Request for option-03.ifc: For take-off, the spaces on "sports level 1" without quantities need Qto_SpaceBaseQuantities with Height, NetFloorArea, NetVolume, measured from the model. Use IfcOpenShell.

First a look at what the model holds.

```python
import ifcopenshell
import ifcopenshell.util.element
import ifcopenshell.util.unit

model = ifcopenshell.open("option-03.ifc")
print(model.schema)
for unit_type in ("LENGTHUNIT", "AREAUNIT", "VOLUMEUNIT"):
    print(unit_type, ifcopenshell.util.unit.calculate_unit_scale(model, unit_type))
storey = next(s for s in model.by_type("IfcBuildingStorey") if s.Name == "sports level 1")
spaces = [e for e in ifcopenshell.util.element.get_decomposition(storey) if e.is_a("IfcSpace")]
for e in sorted(spaces, key=lambda e: e.id()):
    print(e.id(), e.is_a(), e.Name, list(ifcopenshell.util.element.get_psets(e, qtos_only=True)), sep=" | ")
```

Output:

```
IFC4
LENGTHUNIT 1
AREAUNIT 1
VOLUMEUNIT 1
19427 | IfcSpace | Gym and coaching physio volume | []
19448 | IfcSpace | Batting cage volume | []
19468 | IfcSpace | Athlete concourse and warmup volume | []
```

```python
import ifcopenshell
import ifcopenshell.api.pset
import ifcopenshell.geom
import ifcopenshell.util.element
import ifcopenshell.util.shape
import ifcopenshell.util.unit

model = ifcopenshell.open("option-03.ifc")
unit_scale = ifcopenshell.util.unit.calculate_unit_scale(model)
area_scale = ifcopenshell.util.unit.calculate_unit_scale(model, "AREAUNIT")
volume_scale = ifcopenshell.util.unit.calculate_unit_scale(model, "VOLUMEUNIT")
settings = ifcopenshell.geom.settings()

storey = next(s for s in model.by_type("IfcBuildingStorey") if s.Name == "sports level 1")
spaces = [e for e in ifcopenshell.util.element.get_decomposition(storey) if e.is_a("IfcSpace")]

for e in sorted(spaces, key=lambda e: e.id()):
    if ifcopenshell.util.element.get_psets(e, qtos_only=True, should_inherit=False):
        continue
    # Geometry comes back in metres, in the element's own axes.
    shape = ifcopenshell.geom.create_shape(settings, e)
    values = {
        "Height": ifcopenshell.util.shape.get_z(shape.geometry) / unit_scale,
        "NetFloorArea": ifcopenshell.util.shape.get_footprint_area(shape.geometry) / area_scale,
        "NetVolume": ifcopenshell.util.shape.get_volume(shape.geometry) / volume_scale,
    }
    qto = ifcopenshell.api.pset.add_qto(model, product=e, name="Qto_SpaceBaseQuantities")
    ifcopenshell.api.pset.edit_qto(model, qto=qto, properties=values)
    print(e.id(), {k: round(v, 3) for k, v in values.items()})

model.write("option-03_edited.ifc")
```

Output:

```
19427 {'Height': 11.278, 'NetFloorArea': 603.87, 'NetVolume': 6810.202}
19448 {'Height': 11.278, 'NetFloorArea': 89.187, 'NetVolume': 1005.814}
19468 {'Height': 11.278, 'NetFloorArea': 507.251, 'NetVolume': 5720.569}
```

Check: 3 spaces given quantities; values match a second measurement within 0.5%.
